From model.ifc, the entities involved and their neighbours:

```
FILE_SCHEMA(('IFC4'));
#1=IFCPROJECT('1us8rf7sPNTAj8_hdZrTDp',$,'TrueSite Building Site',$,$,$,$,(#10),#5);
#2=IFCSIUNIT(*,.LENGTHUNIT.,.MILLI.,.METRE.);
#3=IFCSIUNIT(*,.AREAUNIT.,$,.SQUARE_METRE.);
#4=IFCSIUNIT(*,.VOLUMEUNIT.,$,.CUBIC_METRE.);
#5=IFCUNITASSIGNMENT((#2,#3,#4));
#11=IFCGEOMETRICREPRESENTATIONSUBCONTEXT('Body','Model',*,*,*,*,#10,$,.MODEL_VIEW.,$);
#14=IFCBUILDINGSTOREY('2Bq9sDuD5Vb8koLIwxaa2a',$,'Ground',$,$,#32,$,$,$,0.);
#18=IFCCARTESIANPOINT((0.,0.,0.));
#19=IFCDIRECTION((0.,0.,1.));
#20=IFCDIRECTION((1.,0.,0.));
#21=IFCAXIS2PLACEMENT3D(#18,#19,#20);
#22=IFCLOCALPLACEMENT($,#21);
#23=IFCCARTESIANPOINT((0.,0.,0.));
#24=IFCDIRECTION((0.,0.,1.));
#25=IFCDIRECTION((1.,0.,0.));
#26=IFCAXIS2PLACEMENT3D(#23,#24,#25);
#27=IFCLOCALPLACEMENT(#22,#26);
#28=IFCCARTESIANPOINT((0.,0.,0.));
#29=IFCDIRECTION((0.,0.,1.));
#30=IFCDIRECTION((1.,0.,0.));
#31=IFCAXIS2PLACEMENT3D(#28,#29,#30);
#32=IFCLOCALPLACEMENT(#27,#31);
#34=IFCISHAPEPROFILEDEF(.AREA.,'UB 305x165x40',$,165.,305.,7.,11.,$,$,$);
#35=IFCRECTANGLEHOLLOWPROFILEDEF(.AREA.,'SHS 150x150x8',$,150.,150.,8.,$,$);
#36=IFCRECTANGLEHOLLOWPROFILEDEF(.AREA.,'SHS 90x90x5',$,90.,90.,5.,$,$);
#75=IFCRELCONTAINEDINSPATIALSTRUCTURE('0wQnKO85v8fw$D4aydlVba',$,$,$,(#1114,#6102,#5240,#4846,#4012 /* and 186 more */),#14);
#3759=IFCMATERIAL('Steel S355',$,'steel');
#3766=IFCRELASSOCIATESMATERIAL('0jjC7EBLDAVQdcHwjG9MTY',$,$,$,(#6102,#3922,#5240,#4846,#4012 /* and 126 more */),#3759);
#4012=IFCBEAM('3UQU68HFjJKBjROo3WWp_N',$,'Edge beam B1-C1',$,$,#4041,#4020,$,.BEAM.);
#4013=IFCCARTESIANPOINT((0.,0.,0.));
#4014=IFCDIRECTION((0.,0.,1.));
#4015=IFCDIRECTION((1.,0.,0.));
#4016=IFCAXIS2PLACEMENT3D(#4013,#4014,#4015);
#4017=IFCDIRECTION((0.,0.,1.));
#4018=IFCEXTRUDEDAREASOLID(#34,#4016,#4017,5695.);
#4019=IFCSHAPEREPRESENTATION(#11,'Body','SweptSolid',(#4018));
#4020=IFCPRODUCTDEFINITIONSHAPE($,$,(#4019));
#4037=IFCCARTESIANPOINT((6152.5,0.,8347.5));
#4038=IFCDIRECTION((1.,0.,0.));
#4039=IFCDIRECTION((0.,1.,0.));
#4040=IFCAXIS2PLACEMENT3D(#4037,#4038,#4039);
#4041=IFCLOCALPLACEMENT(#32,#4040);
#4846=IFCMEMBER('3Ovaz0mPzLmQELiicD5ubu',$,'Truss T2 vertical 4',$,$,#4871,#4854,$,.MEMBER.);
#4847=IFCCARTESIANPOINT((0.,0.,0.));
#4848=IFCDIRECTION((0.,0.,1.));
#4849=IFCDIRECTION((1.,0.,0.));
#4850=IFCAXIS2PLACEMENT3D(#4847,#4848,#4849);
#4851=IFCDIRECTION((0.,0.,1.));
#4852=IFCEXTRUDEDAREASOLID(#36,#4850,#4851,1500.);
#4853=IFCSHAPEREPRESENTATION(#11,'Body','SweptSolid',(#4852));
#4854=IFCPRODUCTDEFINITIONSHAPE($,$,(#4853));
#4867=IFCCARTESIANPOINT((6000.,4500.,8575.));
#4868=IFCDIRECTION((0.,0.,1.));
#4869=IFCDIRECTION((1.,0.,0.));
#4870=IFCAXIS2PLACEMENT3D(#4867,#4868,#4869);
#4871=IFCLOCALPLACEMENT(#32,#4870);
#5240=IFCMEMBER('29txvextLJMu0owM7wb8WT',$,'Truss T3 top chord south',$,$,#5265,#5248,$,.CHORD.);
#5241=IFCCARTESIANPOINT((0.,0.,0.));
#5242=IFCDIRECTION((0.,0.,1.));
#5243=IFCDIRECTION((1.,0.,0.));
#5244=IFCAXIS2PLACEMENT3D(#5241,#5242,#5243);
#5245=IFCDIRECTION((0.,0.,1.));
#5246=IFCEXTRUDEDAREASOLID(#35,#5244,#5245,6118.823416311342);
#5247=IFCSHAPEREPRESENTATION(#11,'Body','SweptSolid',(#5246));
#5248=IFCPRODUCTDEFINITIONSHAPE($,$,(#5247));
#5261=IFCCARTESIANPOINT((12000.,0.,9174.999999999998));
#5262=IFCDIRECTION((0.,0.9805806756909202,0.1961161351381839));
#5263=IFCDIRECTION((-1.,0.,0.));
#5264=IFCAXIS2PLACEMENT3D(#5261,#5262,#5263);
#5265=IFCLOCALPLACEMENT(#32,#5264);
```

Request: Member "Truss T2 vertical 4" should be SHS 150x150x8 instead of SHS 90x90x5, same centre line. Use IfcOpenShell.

```python
import ifcopenshell
import ifcopenshell.util.element
import ifcopenshell.util.representation

model = ifcopenshell.open("model.ifc")

member = model.by_id(4846)
source = next(p for p in model.by_type("IfcRectangleHollowProfileDef") if p.ProfileName == "SHS 150x150x8")

body = ifcopenshell.util.representation.get_representation(member, "Model", "Body")
solid = body.Items[0]
old_profile = solid.SweptArea

# Copy the section's sizes but keep this member's own profile position.
profile = ifcopenshell.util.element.copy(model, source)
profile.Position = old_profile.Position
solid.SweptArea = profile
if not model.get_total_inverses(old_profile):
    ifcopenshell.util.element.remove_deep2(model, old_profile)

print(solid.SweptArea)

model.write("model_v2.ifc")
```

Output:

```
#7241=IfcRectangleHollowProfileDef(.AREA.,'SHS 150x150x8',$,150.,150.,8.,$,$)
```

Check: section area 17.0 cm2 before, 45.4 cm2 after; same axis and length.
